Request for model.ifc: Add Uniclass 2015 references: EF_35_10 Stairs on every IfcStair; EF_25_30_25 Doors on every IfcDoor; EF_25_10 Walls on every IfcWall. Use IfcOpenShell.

First a look at what the model holds.

```python
import ifcopenshell

model = ifcopenshell.open("model.ifc")
print(model.schema)
print("classifications:", [c.Name for c in model.by_type("IfcClassification")])
for ifc_class in ("IfcDoor", "IfcRoof", "IfcStair", "IfcWall", "IfcWindow"):
    print(ifc_class, len(model.by_type(ifc_class)))
```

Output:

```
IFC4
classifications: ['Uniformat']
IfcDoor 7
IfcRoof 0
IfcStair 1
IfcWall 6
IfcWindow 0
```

```python
import ifcopenshell
import ifcopenshell.api.classification

model = ifcopenshell.open("model.ifc")

system = ifcopenshell.api.classification.add_classification(model, classification="Uniclass 2015")

codes = {
    "IfcStair": ("EF_35_10", "Stairs"),
    "IfcDoor": ("EF_25_30_25", "Doors"),
    "IfcWall": ("EF_25_10", "Walls"),
}
for ifc_class, (code, name) in codes.items():
    products = model.by_type(ifc_class)
    ifcopenshell.api.classification.add_reference(
        model, products=products, classification=system, identification=code, name=name
    )
    print(code, len(products))

model.write("model_v2.ifc")
```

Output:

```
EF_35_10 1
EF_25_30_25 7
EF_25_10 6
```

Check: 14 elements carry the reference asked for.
